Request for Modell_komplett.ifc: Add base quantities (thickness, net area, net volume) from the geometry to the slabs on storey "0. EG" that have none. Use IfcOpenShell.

First a look at what the model holds.

```python
import ifcopenshell
import ifcopenshell.util.element
import ifcopenshell.util.unit

model = ifcopenshell.open("Modell_komplett.ifc")
print(model.schema)
for unit_type in ("LENGTHUNIT", "AREAUNIT", "VOLUMEUNIT"):
    print(unit_type, ifcopenshell.util.unit.calculate_unit_scale(model, unit_type))
storey = next(s for s in model.by_type("IfcBuildingStorey") if s.Name == "0. EG")
slabs = [e for e in ifcopenshell.util.element.get_decomposition(storey) if e.is_a("IfcSlab")]
for e in sorted(slabs, key=lambda e: e.id()):
    print(e.id(), e.is_a(), e.Name, list(ifcopenshell.util.element.get_psets(e, qtos_only=True)), sep=" | ")
```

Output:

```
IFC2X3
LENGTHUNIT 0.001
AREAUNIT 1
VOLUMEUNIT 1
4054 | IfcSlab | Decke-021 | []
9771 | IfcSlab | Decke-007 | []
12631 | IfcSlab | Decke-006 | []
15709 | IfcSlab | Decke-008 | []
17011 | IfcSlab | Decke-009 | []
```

```python
import ifcopenshell
import ifcopenshell.api.pset
import ifcopenshell.geom
import ifcopenshell.util.element
import ifcopenshell.util.shape
import ifcopenshell.util.unit

model = ifcopenshell.open("Modell_komplett.ifc")
unit_scale = ifcopenshell.util.unit.calculate_unit_scale(model)
area_scale = ifcopenshell.util.unit.calculate_unit_scale(model, "AREAUNIT")
volume_scale = ifcopenshell.util.unit.calculate_unit_scale(model, "VOLUMEUNIT")
settings = ifcopenshell.geom.settings()

storey = next(s for s in model.by_type("IfcBuildingStorey") if s.Name == "0. EG")
slabs = [e for e in ifcopenshell.util.element.get_decomposition(storey) if e.is_a("IfcSlab")]

for e in sorted(slabs, key=lambda e: e.id()):
    if ifcopenshell.util.element.get_psets(e, qtos_only=True, should_inherit=False):
        continue
    # Geometry comes back in metres, in the element's own axes.
    shape = ifcopenshell.geom.create_shape(settings, e)
    values = {
        "Width": ifcopenshell.util.shape.get_z(shape.geometry) / unit_scale,
        "NetArea": ifcopenshell.util.shape.get_footprint_area(shape.geometry) / area_scale,
        "NetVolume": ifcopenshell.util.shape.get_volume(shape.geometry) / volume_scale,
    }
    qto = ifcopenshell.api.pset.add_qto(model, product=e, name="BaseQuantities")
    ifcopenshell.api.pset.edit_qto(model, qto=qto, properties=values)
    print(e.id(), {k: round(v, 3) for k, v in values.items()})

model.write("Modell_komplett_rev.ifc")
```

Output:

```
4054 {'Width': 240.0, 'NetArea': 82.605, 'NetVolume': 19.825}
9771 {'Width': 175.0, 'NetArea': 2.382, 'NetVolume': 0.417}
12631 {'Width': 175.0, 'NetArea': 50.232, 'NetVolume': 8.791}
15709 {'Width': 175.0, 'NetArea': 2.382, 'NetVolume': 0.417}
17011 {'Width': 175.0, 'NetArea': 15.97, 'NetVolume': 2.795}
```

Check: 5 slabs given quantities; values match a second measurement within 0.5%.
